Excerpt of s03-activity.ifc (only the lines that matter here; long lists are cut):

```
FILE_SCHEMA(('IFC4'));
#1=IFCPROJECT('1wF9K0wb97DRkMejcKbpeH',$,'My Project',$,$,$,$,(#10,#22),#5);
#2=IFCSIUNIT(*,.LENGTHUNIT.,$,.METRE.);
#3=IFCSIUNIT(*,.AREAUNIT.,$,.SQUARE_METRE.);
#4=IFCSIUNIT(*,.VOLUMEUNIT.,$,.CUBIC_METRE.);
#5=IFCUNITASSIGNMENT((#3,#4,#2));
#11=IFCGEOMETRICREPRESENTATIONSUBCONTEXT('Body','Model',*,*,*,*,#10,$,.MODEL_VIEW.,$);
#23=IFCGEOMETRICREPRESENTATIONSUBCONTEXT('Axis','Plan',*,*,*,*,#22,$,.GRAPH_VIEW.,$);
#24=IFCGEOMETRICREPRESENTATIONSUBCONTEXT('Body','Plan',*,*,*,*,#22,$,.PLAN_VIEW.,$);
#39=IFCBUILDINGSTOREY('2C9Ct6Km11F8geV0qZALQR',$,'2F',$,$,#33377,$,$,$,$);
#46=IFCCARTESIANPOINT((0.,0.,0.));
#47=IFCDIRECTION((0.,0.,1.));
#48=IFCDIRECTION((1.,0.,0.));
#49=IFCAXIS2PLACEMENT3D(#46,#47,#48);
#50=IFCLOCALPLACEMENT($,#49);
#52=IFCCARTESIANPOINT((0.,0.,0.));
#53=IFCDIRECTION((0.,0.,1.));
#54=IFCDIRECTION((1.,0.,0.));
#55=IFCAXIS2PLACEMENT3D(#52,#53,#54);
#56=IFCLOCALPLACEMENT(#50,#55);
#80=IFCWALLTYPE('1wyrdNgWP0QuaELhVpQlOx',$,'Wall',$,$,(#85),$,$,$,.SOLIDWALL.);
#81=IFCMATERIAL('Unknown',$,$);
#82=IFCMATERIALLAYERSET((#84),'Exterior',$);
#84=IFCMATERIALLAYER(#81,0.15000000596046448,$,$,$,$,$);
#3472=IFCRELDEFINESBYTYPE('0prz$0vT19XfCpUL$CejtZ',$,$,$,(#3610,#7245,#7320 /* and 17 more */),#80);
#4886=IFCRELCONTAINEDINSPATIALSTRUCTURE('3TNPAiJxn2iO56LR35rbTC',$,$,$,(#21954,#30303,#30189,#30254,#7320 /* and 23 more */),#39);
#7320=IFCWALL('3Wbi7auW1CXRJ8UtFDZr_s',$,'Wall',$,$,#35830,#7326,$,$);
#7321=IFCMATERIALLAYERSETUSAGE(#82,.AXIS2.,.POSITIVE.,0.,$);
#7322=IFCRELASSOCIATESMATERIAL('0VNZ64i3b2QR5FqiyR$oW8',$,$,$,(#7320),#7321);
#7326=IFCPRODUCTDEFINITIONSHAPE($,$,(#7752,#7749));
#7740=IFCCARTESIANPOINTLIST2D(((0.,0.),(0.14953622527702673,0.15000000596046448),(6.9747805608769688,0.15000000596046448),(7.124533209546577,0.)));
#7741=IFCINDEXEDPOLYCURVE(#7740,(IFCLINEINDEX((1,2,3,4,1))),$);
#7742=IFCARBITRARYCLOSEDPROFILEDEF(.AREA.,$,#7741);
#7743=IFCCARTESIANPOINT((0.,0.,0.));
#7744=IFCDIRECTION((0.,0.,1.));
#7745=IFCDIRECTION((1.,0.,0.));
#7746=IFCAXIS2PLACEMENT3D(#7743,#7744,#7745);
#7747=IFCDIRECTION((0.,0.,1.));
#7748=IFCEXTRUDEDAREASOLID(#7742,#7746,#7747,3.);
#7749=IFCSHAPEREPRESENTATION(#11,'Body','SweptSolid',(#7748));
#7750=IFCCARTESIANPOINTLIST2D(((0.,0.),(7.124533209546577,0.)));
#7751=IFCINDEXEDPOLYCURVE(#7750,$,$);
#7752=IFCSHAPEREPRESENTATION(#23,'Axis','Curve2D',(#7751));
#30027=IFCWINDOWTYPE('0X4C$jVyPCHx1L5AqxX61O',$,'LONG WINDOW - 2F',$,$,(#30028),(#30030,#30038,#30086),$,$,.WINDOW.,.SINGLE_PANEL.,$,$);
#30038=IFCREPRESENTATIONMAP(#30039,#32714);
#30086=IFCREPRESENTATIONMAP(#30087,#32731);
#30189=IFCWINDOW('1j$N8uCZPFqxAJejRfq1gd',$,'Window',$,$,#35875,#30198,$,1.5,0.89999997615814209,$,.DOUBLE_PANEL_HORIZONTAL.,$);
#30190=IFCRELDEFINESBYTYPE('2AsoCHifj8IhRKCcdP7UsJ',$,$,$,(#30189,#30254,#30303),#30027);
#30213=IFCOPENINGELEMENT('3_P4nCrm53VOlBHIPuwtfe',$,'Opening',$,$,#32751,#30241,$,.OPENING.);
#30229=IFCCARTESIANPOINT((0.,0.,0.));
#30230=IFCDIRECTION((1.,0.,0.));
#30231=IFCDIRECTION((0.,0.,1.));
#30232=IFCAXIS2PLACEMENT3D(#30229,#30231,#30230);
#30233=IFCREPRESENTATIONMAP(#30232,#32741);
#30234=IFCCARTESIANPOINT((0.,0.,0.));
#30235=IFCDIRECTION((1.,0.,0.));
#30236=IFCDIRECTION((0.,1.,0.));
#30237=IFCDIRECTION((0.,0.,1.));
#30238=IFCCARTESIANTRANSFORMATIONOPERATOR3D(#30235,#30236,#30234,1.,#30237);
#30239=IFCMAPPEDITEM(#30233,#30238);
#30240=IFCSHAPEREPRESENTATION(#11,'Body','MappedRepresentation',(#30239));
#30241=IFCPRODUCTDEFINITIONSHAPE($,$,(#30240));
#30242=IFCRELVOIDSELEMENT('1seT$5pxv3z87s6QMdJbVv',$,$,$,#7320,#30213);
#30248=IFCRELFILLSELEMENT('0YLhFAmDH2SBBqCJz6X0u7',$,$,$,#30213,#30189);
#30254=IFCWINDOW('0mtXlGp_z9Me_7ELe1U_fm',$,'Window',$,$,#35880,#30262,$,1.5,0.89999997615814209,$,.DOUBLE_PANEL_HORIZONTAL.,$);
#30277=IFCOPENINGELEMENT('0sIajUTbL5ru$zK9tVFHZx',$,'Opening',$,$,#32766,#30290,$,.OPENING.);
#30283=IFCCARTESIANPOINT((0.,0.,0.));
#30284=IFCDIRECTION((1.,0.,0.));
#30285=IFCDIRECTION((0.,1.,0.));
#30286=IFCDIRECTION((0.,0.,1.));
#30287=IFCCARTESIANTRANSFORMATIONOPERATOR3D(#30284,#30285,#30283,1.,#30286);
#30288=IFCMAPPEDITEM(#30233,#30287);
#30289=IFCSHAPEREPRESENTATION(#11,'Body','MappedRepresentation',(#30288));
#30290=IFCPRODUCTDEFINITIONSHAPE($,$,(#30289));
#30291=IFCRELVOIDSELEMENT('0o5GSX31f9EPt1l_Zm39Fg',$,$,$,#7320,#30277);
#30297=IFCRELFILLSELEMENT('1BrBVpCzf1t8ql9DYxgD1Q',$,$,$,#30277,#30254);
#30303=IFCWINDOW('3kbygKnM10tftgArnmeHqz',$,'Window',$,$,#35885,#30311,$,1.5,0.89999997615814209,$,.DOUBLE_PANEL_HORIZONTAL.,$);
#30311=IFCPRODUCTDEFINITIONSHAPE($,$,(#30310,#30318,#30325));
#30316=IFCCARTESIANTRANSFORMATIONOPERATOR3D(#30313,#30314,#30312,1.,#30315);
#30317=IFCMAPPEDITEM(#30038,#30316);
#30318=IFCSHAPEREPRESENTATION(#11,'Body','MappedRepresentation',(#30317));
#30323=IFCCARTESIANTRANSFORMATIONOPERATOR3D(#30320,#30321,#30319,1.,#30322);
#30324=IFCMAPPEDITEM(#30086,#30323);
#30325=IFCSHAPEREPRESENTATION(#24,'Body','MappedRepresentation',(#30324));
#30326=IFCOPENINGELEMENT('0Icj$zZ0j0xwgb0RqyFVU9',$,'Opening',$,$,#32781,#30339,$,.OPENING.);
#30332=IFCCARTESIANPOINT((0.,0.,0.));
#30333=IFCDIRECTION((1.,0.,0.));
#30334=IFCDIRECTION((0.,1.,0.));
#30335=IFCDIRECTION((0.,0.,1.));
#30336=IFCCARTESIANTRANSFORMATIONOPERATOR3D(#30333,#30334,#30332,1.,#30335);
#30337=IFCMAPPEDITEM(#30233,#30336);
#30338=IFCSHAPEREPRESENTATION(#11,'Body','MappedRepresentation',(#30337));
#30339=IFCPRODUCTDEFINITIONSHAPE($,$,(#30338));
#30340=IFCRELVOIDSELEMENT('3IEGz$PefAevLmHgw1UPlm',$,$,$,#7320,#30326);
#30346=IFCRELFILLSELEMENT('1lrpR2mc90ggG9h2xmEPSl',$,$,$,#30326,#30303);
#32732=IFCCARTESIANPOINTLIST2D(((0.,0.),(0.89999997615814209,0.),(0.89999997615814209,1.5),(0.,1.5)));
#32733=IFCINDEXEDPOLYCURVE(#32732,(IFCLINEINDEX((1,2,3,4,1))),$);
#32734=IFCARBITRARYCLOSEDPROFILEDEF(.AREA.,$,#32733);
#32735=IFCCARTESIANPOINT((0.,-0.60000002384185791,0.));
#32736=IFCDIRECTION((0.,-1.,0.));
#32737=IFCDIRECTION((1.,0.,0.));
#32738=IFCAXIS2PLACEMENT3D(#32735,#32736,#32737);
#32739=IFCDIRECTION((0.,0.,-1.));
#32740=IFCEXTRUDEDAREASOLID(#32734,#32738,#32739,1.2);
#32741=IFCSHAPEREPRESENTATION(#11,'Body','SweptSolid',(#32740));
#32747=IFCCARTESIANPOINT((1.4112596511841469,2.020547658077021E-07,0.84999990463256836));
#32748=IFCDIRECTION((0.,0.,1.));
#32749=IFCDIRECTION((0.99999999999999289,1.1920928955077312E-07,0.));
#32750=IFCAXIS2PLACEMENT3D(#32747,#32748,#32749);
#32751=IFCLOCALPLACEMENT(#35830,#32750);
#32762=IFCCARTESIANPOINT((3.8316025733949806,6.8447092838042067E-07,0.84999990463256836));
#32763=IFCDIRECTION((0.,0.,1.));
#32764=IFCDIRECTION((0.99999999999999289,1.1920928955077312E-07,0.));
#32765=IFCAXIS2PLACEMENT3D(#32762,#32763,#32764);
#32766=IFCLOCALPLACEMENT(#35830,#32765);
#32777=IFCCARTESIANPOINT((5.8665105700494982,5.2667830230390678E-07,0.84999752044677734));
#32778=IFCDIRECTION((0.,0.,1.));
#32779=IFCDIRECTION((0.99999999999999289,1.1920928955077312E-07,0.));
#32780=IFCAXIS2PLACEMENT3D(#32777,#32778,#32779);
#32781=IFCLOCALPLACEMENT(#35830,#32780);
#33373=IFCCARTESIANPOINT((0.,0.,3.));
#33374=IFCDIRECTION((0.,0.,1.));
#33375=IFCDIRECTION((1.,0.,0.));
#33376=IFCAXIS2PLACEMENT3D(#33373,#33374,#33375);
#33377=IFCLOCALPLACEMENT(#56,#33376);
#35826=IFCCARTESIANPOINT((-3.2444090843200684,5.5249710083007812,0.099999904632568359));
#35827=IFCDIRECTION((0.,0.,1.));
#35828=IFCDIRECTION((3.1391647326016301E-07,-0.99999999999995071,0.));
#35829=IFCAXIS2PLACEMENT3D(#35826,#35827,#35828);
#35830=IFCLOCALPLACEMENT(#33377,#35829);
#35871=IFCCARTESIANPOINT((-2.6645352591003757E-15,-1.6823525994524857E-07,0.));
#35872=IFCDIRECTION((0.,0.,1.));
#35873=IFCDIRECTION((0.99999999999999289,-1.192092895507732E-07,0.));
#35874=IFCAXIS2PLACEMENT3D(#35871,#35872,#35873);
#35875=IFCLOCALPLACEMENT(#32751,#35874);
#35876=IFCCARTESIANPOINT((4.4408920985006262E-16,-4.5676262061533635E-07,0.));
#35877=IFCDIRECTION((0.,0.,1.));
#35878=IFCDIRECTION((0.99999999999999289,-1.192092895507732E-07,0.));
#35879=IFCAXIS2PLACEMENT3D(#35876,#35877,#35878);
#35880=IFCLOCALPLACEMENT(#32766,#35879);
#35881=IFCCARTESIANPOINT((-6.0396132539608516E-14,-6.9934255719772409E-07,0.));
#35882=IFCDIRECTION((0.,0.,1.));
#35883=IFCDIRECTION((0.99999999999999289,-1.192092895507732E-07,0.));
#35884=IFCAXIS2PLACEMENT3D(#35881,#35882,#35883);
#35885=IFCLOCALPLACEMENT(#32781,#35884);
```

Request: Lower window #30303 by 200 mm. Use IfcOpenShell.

```python
import numpy as np
import ifcopenshell
import ifcopenshell.api.geometry
import ifcopenshell.util.placement
import ifcopenshell.util.unit

model = ifcopenshell.open("s03-activity.ifc")
unit_scale = ifcopenshell.util.unit.calculate_unit_scale(model)

window = model.by_guid("3kbygKnM10tftgArnmeHqz")
opening = window.FillsVoids[0].RelatingOpeningElement
dz = -0.2 / unit_scale

shift = np.array([0.0, 0.0, dz])
# The window is placed relative to its opening, so it follows when the opening moves.
matrix = ifcopenshell.util.placement.get_local_placement(opening.ObjectPlacement)
matrix[:3, 3] += shift
ifcopenshell.api.geometry.edit_object_placement(
    model, product=opening, matrix=matrix, is_si=False, should_transform_children=True
)

print(f"moved by {dz * unit_scale:+.3f} m")

model.write("s03-activity-out.ifc")
```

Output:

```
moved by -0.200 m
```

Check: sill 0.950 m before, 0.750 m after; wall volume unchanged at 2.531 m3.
